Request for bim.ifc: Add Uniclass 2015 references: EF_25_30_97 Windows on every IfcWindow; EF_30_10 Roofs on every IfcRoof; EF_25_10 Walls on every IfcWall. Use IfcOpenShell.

First a look at what the model holds.

```python
import ifcopenshell

model = ifcopenshell.open("bim.ifc")
print(model.schema)
print("classifications:", [c.Name for c in model.by_type("IfcClassification")])
for ifc_class in ("IfcDoor", "IfcRoof", "IfcStair", "IfcWall", "IfcWindow"):
    print(ifc_class, len(model.by_type(ifc_class)))
```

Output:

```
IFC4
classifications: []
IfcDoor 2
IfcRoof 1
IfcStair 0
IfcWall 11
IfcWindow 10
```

```python
import ifcopenshell
import ifcopenshell.api.classification

model = ifcopenshell.open("bim.ifc")

system = ifcopenshell.api.classification.add_classification(model, classification="Uniclass 2015")

codes = {
    "IfcWindow": ("EF_25_30_97", "Windows"),
    "IfcRoof": ("EF_30_10", "Roofs"),
    "IfcWall": ("EF_25_10", "Walls"),
}
for ifc_class, (code, name) in codes.items():
    products = model.by_type(ifc_class)
    ifcopenshell.api.classification.add_reference(
        model, products=products, classification=system, identification=code, name=name
    )
    print(code, len(products))

model.write("bim_updated.ifc")
```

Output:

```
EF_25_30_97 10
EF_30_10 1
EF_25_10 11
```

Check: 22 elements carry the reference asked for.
